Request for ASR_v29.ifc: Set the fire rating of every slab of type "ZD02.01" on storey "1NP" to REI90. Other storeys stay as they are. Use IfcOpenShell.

First a look at what the model holds.

```python
import ifcopenshell
import ifcopenshell.util.element

model = ifcopenshell.open("ASR_v29.ifc")
print(model.schema)
storey = next(s for s in model.by_type("IfcBuildingStorey") if s.Name == "1NP")
slabs = [e for e in ifcopenshell.util.element.get_decomposition(storey) if e.is_a("IfcSlab")]
seen = {}
for e in slabs:
    element_type = ifcopenshell.util.element.get_type(e)
    key = (element_type.Name if element_type != e and element_type else None, ifcopenshell.util.element.get_pset(e, "Pset_SlabCommon", "FireRating"))
    seen[key] = seen.get(key, 0) + 1
for (name, value), count in sorted(seen.items(), key=str):
    print(count, "x", name, "|", value)
```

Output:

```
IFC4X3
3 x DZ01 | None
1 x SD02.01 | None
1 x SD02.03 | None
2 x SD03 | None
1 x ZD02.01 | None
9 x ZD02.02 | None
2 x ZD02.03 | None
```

```python
import ifcopenshell
import ifcopenshell.api.pset
import ifcopenshell.util.element

model = ifcopenshell.open("ASR_v29.ifc")

storey = next(s for s in model.by_type("IfcBuildingStorey") if s.Name == "1NP")
slabs = [e for e in ifcopenshell.util.element.get_decomposition(storey) if e.is_a("IfcSlab")]

count = 0
for e in slabs:
    element_type = ifcopenshell.util.element.get_type(e)
    if element_type in (None, e) or element_type.Name != "ZD02.01":
        continue
    # add_pset returns the element's existing set when there is one.
    pset = ifcopenshell.api.pset.add_pset(model, product=e, name="Pset_SlabCommon")
    ifcopenshell.api.pset.edit_pset(model, pset=pset, properties={"FireRating": "REI90"})
    count += 1

print(count, "slabs updated")

model.write("ASR_v29-out.ifc")
```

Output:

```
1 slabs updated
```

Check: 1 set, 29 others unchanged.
